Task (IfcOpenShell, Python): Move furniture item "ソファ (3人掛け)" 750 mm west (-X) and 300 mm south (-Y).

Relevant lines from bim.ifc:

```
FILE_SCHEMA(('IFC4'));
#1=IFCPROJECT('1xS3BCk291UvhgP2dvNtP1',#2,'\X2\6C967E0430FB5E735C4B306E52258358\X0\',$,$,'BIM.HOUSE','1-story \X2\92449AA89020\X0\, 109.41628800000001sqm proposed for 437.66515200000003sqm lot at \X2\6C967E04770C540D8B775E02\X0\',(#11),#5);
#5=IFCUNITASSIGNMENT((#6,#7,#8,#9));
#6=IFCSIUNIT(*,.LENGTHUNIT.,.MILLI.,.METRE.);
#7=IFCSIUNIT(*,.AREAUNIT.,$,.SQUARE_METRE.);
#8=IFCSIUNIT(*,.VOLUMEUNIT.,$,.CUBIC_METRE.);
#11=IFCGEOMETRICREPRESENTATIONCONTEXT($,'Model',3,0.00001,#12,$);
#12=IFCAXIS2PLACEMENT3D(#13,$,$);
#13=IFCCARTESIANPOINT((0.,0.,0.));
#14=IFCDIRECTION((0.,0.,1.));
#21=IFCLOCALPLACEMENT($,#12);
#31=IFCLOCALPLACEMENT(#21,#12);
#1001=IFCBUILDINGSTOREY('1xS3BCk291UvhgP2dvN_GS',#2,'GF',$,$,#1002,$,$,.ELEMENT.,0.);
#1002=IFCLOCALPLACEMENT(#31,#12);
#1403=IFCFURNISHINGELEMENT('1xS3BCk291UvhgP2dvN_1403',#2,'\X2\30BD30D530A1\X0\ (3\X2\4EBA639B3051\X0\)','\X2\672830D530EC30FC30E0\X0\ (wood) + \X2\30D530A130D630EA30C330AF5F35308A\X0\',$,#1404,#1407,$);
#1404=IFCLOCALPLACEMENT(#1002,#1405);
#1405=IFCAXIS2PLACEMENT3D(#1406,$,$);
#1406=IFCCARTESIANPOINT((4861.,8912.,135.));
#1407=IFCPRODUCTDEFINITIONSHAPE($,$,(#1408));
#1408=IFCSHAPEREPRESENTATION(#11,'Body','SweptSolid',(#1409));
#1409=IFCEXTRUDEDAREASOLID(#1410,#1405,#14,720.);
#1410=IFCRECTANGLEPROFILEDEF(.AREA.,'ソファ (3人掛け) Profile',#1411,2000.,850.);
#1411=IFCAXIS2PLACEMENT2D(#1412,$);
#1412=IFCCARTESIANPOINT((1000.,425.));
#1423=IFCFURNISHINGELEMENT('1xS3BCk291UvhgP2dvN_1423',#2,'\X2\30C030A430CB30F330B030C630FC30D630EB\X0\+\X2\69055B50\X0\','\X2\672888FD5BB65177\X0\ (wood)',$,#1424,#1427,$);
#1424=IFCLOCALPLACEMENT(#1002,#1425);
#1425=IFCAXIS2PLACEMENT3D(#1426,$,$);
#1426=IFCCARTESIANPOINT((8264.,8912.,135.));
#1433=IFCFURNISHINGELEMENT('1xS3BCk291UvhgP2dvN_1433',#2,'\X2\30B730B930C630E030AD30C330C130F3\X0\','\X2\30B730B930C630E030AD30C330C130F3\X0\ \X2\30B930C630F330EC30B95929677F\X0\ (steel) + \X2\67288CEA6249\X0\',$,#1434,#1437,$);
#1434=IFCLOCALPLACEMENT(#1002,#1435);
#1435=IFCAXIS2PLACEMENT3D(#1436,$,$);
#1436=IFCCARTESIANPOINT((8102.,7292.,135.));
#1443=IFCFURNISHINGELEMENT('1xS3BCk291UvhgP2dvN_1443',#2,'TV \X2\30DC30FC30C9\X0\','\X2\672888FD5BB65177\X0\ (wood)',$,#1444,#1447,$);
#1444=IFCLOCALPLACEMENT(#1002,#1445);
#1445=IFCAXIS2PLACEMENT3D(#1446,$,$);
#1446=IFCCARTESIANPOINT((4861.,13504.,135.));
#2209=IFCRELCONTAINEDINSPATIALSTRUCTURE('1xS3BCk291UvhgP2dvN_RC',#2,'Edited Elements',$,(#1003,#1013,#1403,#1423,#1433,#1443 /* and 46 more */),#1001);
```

```python
import ifcopenshell
import ifcopenshell.api.geometry
import ifcopenshell.util.placement
import ifcopenshell.util.unit

model = ifcopenshell.open("bim.ifc")
unit_scale = ifcopenshell.util.unit.calculate_unit_scale(model)

item = model.by_id(1403)
matrix = ifcopenshell.util.placement.get_local_placement(item.ObjectPlacement)
matrix[0, 3] -= 0.75 / unit_scale
matrix[1, 3] -= 0.3 / unit_scale
ifcopenshell.api.geometry.edit_object_placement(model, product=item, matrix=matrix, is_si=False)

print(ifcopenshell.util.placement.get_local_placement(item.ObjectPlacement).round(3) + 0.0)

model.write("bim_updated.ifc")
```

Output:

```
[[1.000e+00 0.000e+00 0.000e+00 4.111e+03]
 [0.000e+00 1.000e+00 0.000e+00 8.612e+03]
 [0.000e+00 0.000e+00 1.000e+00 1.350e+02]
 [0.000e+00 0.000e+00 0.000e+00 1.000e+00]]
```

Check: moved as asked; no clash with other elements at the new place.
